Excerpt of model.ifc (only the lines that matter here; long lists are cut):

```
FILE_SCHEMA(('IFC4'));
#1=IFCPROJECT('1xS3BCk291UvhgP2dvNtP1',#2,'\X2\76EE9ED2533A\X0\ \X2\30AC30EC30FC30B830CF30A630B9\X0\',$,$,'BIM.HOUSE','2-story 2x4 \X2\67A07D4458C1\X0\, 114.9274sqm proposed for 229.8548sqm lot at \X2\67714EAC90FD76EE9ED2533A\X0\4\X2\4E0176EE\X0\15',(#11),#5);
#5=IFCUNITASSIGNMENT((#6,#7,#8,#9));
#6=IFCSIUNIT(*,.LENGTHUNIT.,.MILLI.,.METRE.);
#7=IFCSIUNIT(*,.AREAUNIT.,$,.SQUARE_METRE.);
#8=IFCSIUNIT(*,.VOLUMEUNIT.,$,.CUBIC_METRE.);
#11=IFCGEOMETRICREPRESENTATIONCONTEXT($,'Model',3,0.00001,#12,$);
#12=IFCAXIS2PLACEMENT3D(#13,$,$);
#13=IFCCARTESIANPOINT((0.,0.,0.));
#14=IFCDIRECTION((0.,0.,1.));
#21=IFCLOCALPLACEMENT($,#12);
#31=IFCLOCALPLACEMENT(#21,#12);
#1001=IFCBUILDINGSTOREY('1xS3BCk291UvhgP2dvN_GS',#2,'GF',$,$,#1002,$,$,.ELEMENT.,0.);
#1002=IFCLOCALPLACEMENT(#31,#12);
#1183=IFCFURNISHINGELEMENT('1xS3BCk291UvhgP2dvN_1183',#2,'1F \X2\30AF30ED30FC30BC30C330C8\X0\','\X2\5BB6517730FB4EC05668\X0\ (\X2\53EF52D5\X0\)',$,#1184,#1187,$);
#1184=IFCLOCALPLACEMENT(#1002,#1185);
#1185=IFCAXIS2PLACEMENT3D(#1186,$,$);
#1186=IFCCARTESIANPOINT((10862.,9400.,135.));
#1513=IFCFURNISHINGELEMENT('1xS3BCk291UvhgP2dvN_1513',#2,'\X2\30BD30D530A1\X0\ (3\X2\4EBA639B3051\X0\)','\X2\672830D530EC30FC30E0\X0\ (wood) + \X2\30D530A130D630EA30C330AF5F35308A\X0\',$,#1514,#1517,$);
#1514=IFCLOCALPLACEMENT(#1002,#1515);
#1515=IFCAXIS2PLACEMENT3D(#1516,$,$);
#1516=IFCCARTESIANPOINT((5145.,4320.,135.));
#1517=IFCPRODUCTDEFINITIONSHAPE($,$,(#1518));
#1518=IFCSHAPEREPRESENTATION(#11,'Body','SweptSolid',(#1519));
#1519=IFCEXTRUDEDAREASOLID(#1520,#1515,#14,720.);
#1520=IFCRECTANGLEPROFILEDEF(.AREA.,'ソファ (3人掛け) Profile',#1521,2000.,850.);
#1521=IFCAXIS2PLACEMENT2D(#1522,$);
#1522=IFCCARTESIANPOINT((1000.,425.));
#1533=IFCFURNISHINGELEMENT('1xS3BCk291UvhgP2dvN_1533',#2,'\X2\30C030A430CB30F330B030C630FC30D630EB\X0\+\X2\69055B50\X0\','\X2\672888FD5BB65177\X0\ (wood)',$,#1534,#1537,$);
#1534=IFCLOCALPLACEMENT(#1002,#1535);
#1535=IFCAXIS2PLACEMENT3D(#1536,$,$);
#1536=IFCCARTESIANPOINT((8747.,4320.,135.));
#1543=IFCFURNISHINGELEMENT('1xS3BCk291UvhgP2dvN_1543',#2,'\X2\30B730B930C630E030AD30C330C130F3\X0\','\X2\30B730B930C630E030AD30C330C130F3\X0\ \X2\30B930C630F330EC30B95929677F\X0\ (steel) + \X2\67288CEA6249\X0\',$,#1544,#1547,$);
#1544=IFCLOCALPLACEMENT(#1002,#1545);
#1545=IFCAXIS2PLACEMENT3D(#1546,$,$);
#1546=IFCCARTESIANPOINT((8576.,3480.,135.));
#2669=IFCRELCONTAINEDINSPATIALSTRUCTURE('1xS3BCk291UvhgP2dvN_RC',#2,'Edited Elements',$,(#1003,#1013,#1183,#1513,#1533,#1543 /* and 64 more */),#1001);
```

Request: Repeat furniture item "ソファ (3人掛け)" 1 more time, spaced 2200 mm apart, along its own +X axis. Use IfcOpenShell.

```python
import ifcopenshell
import ifcopenshell.api.geometry
import ifcopenshell.api.root
import ifcopenshell.util.element
import ifcopenshell.util.placement
import ifcopenshell.util.unit

model = ifcopenshell.open("model.ifc")
unit_scale = ifcopenshell.util.unit.calculate_unit_scale(model)


def reuse_history(source, copy):
    """copy_class also copies each property set's owner history, people and application; keep the originals."""
    for rel in copy.IsDefinedBy:
        if rel.is_a("IfcRelDefinesByProperties") and (history := rel.RelatingPropertyDefinition.OwnerHistory):
            rel.RelatingPropertyDefinition.OwnerHistory = source.OwnerHistory
            ifcopenshell.util.element.remove_deep2(model, history)


source = model.by_id(1513)
base = ifcopenshell.util.placement.get_local_placement(source.ObjectPlacement)
step = base[:3, 0] * 2.2 / unit_scale

for i in range(1, 2):
    copy = ifcopenshell.api.root.copy_class(model, product=source)
    copy.Representation = ifcopenshell.util.element.copy_deep(
        model, source.Representation, exclude=["IfcGeometricRepresentationContext", "IfcRepresentationMap"]
    )
    reuse_history(source, copy)
    matrix = base.copy()
    matrix[:3, 3] += i * step
    print("added at", matrix[:3, 3].round(3) + 0.0)
    ifcopenshell.api.geometry.edit_object_placement(model, product=copy, matrix=matrix, is_si=False)

model.write("model_rev.ifc")
```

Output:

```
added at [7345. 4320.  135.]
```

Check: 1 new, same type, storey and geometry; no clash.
